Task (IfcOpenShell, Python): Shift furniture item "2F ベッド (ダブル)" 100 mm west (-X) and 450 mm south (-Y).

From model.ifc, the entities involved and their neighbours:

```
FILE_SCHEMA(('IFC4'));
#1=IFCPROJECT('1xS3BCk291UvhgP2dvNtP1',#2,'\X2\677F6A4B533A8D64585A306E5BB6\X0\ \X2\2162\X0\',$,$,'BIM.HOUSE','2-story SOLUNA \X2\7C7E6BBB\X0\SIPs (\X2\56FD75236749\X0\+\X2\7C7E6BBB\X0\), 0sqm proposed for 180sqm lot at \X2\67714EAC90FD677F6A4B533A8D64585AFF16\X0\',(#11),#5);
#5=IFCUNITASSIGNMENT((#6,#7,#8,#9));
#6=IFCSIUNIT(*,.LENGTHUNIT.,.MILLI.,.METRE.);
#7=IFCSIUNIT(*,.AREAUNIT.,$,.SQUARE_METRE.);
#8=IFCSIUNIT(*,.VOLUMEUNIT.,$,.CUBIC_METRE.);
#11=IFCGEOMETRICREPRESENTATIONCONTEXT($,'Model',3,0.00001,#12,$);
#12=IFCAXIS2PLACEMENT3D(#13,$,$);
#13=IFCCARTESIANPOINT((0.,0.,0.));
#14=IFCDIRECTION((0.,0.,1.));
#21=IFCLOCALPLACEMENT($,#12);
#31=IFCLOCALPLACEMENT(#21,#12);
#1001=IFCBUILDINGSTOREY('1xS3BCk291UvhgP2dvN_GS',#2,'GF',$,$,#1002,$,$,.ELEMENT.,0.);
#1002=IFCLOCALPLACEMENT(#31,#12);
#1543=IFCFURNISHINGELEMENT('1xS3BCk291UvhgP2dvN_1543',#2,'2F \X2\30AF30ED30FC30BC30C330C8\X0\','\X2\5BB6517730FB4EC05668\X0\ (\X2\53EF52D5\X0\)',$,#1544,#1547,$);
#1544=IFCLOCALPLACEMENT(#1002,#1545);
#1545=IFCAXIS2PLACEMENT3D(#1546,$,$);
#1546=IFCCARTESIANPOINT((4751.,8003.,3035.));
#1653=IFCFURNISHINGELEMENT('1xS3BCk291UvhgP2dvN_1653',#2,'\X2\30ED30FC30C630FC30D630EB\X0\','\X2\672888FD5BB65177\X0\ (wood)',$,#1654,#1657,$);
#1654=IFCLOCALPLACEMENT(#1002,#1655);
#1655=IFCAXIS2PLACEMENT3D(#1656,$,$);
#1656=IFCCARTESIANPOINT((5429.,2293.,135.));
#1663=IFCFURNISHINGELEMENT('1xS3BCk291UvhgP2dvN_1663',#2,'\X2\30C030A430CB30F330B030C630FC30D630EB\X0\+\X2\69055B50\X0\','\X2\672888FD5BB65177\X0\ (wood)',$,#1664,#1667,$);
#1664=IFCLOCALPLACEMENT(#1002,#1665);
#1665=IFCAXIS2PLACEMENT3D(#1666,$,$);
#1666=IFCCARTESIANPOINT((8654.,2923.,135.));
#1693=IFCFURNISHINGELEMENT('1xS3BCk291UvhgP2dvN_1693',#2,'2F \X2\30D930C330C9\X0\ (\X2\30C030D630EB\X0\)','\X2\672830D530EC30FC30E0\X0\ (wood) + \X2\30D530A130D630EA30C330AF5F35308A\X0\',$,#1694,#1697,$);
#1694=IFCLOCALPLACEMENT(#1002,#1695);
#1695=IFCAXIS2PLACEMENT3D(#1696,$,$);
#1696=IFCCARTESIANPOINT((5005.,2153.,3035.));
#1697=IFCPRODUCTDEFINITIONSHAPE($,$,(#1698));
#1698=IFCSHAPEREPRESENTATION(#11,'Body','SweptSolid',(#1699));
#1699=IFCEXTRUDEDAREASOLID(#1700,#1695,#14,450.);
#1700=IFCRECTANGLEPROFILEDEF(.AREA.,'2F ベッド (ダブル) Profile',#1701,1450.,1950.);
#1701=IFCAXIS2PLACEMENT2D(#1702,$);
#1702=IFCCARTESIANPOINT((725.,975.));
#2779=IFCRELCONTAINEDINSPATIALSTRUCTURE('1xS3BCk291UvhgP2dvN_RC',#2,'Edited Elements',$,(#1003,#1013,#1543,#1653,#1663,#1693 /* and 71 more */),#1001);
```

```python
import ifcopenshell
import ifcopenshell.api.geometry
import ifcopenshell.util.placement

model = ifcopenshell.open("model.ifc")

item = model.by_guid("1xS3BCk291UvhgP2dvN_1693")
matrix = ifcopenshell.util.placement.get_local_placement(item.ObjectPlacement)
matrix[0, 3] -= 100.0
matrix[1, 3] -= 450.0
ifcopenshell.api.geometry.edit_object_placement(model, product=item, matrix=matrix, is_si=False)

print(ifcopenshell.util.placement.get_local_placement(item.ObjectPlacement).round(3) + 0.0)

model.write("model_edited.ifc")
```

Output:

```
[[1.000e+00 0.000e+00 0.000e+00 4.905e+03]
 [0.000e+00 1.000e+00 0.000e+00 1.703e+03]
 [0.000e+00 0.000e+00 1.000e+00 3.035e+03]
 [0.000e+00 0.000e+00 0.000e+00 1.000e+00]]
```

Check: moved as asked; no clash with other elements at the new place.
